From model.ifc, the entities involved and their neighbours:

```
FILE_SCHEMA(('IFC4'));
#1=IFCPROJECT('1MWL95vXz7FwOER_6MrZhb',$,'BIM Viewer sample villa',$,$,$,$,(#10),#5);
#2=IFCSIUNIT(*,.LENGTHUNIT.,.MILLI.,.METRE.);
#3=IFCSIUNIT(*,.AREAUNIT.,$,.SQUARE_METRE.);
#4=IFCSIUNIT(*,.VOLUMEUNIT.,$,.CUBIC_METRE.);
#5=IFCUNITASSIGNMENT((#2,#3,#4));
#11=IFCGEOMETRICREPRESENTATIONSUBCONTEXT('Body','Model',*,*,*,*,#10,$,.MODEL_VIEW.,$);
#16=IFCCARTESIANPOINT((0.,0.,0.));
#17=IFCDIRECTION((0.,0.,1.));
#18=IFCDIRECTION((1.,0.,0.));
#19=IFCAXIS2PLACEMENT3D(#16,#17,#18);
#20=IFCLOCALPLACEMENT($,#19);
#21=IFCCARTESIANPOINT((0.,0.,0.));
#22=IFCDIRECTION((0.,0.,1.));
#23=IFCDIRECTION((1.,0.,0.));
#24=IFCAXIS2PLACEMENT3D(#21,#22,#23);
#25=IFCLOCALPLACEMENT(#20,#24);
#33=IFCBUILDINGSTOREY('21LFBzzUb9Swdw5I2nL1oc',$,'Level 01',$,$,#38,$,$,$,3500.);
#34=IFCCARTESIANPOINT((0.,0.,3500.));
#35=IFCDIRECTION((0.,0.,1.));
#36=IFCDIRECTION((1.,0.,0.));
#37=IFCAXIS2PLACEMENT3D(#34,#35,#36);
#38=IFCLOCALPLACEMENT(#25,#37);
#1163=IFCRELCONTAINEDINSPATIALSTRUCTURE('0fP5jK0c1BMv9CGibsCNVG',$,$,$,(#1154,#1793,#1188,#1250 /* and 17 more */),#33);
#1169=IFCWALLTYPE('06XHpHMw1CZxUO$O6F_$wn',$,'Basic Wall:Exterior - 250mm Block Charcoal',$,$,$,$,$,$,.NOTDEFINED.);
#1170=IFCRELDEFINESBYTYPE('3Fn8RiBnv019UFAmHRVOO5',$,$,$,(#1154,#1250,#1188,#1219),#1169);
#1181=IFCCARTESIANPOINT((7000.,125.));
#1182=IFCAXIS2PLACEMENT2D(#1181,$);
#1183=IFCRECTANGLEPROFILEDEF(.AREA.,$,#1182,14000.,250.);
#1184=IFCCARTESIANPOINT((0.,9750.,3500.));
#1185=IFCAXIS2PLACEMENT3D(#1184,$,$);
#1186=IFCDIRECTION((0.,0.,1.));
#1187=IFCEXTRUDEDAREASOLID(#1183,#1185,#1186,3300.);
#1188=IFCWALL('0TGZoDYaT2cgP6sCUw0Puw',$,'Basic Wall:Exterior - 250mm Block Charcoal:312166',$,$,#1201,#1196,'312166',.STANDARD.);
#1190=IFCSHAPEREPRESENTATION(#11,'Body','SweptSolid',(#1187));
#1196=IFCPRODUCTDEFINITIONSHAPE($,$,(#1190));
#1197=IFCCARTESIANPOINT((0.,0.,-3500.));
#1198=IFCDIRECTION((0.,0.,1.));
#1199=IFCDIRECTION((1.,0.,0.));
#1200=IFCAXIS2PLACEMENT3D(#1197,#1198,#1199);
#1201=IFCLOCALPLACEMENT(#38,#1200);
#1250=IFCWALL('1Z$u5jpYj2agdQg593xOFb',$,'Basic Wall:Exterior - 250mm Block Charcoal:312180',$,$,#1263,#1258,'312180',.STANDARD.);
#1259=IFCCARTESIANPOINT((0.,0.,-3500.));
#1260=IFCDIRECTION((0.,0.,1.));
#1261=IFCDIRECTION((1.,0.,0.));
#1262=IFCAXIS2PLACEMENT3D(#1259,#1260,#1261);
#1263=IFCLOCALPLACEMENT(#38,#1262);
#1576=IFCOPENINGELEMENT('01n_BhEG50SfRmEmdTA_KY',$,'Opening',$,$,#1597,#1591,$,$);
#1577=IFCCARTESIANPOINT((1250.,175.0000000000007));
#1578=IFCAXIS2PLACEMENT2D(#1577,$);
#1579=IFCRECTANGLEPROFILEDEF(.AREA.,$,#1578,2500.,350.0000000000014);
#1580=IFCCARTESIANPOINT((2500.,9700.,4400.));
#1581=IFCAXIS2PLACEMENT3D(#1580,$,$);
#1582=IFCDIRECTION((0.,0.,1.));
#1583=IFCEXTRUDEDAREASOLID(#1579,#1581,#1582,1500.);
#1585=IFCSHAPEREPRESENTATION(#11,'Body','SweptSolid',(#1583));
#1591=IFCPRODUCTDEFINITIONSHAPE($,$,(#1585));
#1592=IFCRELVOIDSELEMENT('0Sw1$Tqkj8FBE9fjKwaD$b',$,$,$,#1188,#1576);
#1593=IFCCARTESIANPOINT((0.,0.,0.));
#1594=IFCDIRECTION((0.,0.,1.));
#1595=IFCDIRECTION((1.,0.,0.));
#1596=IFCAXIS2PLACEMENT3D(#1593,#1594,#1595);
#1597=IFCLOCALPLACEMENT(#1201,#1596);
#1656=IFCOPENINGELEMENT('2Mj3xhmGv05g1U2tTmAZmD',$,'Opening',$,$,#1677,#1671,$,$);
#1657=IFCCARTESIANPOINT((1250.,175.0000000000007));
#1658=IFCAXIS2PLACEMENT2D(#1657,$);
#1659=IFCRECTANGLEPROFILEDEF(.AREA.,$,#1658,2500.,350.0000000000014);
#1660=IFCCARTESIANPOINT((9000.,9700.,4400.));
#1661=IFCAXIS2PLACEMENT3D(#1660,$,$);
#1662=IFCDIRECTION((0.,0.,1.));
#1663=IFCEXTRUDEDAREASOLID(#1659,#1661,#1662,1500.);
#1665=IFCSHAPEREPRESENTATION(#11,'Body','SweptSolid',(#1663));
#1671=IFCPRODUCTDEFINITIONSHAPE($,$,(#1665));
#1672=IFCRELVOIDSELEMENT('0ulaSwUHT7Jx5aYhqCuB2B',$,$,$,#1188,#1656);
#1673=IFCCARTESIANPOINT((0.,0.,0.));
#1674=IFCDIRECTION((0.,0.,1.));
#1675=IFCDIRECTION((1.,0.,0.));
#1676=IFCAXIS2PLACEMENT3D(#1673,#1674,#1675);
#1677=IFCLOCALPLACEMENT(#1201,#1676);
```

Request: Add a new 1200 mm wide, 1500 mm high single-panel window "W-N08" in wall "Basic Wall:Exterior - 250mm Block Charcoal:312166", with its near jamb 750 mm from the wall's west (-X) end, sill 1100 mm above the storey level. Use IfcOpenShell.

```python
import numpy as np
import ifcopenshell
import ifcopenshell.api.feature
import ifcopenshell.api.geometry
import ifcopenshell.api.root
import ifcopenshell.api.spatial
import ifcopenshell.geom
import ifcopenshell.util.element
import ifcopenshell.util.placement
import ifcopenshell.util.representation
import ifcopenshell.util.shape
import ifcopenshell.util.unit

model = ifcopenshell.open("model.ifc")
unit_scale = ifcopenshell.util.unit.calculate_unit_scale(model)
settings = ifcopenshell.geom.settings()


def volume(element):
    """Net volume in cubic metres, openings subtracted."""
    shape = ifcopenshell.geom.create_shape(settings, element)
    return ifcopenshell.util.shape.get_volume(shape.geometry)


wall = model.by_guid("0TGZoDYaT2cgP6sCUw0Puw")
storey = ifcopenshell.util.element.get_container(wall, ifc_class="IfcBuildingStorey")
context = ifcopenshell.util.representation.get_context(model, "Model", "Body", "MODEL_VIEW")
before = volume(wall)

width, height, from_end, sill = 1.2, 1.5, 0.75, 1.1  # metres

# The wall runs along its own X axis, and the end named is its -X end.
wall_shape = ifcopenshell.geom.create_shape(settings, wall)
x, y, z = ifcopenshell.util.shape.get_vertices(wall_shape.geometry).T
start = x.min() + from_end
face, thickness = float(y.min()), float(y.max() - y.min())
wall_matrix = ifcopenshell.util.placement.get_local_placement(wall.ObjectPlacement)
level = ifcopenshell.util.placement.get_local_placement(storey.ObjectPlacement)[2, 3]


def in_wall(x, y):
    """Placement at x, y metres in the wall's axes, at sill height."""
    matrix = wall_matrix.copy()
    matrix[:, 3] = wall_matrix @ np.array([x / unit_scale, y / unit_scale, 0.0, 1.0])
    matrix[2, 3] = level + sill / unit_scale
    return matrix


# Opening: a box that overshoots both wall faces by 50 mm.
opening = ifcopenshell.api.root.create_entity(model, ifc_class="IfcOpeningElement", predefined_type="OPENING")
box = ifcopenshell.api.geometry.add_wall_representation(
    model, context=context, length=width, height=height, thickness=thickness + 0.1
)
ifcopenshell.api.geometry.assign_representation(model, product=opening, representation=box)
ifcopenshell.api.geometry.edit_object_placement(model, product=opening, matrix=in_wall(start, face - 0.05), is_si=False)
ifcopenshell.api.feature.add_feature(model, feature=opening, element=wall)

window = ifcopenshell.api.root.create_entity(model, ifc_class="IfcWindow", name="W-N08", predefined_type="WINDOW")
window.OverallWidth, window.OverallHeight = width / unit_scale, height / unit_scale
window.PartitioningType = "SINGLE_PANEL"
body = ifcopenshell.api.geometry.add_window_representation(
    model,
    context=context,
    overall_width=window.OverallWidth,
    overall_height=window.OverallHeight,
    partition_type="SINGLE_PANEL",
)
ifcopenshell.api.geometry.assign_representation(model, product=window, representation=body)
ifcopenshell.api.spatial.assign_container(model, products=[window], relating_structure=storey)
ifcopenshell.api.feature.add_filling(model, opening=opening, element=window)

# Centre the window in the wall's thickness.
ifcopenshell.api.geometry.edit_object_placement(model, product=window, matrix=in_wall(start, face), is_si=False)
window_shape = ifcopenshell.geom.create_shape(settings, window)
depth = ifcopenshell.util.shape.get_vertices(window_shape.geometry)[:, 1]
offset = face + thickness / 2 - (depth.min() + depth.max()) / 2
ifcopenshell.api.geometry.edit_object_placement(model, product=window, matrix=in_wall(start, offset), is_si=False)

after = volume(wall)

print(f"wall volume {before:.3f} -> {after:.3f} m3")

model.write("model_updated.ifc")
```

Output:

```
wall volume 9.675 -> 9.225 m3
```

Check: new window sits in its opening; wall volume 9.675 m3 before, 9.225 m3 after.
